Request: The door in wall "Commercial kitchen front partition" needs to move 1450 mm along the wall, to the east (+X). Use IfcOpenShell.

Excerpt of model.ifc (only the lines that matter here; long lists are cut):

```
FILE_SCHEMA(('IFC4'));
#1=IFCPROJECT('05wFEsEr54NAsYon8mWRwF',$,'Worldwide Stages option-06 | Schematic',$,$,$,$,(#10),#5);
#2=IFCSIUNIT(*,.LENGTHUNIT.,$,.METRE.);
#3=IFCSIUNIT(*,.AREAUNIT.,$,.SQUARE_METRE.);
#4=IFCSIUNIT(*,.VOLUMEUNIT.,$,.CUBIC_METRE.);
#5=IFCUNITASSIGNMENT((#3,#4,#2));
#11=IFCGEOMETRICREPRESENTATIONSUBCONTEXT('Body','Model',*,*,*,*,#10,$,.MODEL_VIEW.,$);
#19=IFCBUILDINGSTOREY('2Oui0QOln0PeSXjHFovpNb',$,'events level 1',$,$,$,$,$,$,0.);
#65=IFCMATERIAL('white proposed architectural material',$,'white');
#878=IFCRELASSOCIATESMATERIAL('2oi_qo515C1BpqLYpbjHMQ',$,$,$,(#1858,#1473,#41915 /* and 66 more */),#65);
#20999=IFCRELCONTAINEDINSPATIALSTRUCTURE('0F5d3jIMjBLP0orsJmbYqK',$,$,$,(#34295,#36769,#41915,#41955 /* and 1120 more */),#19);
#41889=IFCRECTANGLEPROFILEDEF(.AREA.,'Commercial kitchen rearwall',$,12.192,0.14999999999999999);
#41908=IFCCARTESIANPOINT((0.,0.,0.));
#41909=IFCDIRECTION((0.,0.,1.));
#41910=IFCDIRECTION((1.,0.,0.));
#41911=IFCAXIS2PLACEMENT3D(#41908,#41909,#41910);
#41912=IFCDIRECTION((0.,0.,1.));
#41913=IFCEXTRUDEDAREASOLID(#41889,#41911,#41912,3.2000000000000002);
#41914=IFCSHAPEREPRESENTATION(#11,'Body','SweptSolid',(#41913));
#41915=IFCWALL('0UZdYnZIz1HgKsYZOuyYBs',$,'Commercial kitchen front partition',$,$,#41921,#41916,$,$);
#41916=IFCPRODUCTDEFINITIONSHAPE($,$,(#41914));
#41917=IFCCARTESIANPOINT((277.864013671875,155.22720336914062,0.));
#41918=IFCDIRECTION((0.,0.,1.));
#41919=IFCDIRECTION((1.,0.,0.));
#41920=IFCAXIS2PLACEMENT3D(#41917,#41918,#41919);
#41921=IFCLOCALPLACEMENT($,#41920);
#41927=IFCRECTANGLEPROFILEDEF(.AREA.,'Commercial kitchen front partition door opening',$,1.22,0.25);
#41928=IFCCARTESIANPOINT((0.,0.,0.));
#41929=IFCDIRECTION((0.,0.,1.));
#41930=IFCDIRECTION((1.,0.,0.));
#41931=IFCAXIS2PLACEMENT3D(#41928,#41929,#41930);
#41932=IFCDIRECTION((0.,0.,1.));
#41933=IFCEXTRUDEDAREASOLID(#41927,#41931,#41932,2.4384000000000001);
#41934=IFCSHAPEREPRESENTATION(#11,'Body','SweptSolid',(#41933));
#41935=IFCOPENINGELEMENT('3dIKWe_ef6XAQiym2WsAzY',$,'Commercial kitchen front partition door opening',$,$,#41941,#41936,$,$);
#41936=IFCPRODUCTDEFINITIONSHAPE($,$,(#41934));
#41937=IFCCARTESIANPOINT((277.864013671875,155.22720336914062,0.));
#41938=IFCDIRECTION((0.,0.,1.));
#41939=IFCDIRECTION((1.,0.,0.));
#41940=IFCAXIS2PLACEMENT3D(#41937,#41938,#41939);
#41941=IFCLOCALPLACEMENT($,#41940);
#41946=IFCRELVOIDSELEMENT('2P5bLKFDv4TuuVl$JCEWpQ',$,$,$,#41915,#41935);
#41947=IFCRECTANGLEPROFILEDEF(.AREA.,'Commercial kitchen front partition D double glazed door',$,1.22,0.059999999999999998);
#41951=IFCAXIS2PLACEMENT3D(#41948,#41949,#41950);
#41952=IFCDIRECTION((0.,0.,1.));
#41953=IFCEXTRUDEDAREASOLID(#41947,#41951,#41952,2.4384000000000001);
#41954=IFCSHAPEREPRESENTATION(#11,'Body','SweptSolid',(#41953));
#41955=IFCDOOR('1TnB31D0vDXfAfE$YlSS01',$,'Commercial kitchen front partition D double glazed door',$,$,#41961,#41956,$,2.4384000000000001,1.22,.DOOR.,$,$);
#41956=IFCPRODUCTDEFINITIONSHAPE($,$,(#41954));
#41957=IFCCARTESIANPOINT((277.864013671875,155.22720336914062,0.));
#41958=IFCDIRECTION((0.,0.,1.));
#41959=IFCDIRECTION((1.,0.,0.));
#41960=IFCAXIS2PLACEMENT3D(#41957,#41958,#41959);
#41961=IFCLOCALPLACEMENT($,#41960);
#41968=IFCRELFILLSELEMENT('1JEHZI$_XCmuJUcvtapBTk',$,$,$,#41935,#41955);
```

```python
import ifcopenshell
import ifcopenshell.api.geometry
import ifcopenshell.util.placement
import ifcopenshell.util.unit

model = ifcopenshell.open("model.ifc")
unit_scale = ifcopenshell.util.unit.calculate_unit_scale(model)

door = model.by_guid("1TnB31D0vDXfAfE$YlSS01")
opening = door.FillsVoids[0].RelatingOpeningElement
wall = opening.VoidsElements[0].RelatingBuildingElement

wall_matrix = ifcopenshell.util.placement.get_local_placement(wall.ObjectPlacement)
shift = wall_matrix[:3, 0] * 1.45 / unit_scale
before = ifcopenshell.util.placement.get_local_placement(door.ObjectPlacement)[:3, 3].copy()

# The door is not placed relative to its opening, so move both.
for product in (opening, door):
    matrix = ifcopenshell.util.placement.get_local_placement(product.ObjectPlacement)
    matrix[:3, 3] += shift
    ifcopenshell.api.geometry.edit_object_placement(model, product=product, matrix=matrix, is_si=False)

after = ifcopenshell.util.placement.get_local_placement(door.ObjectPlacement)[:3, 3]
print("door moved by", (after - before).round(3) + 0.0)

model.write("model_rev.ifc")
```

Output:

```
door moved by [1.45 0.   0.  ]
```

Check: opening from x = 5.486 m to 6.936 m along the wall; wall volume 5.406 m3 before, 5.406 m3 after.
